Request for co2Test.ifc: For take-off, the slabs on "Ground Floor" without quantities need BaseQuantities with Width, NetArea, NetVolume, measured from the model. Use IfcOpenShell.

First a look at what the model holds.

```python
import ifcopenshell
import ifcopenshell.util.element
import ifcopenshell.util.unit

model = ifcopenshell.open("co2Test.ifc")
print(model.schema)
for unit_type in ("LENGTHUNIT", "AREAUNIT", "VOLUMEUNIT"):
    print(unit_type, ifcopenshell.util.unit.calculate_unit_scale(model, unit_type))
storey = next(s for s in model.by_type("IfcBuildingStorey") if s.Name == "Ground Floor")
slabs = [e for e in ifcopenshell.util.element.get_decomposition(storey) if e.is_a("IfcSlab")]
for e in sorted(slabs, key=lambda e: e.id()):
    print(e.id(), e.is_a(), e.Name, list(ifcopenshell.util.element.get_psets(e, qtos_only=True)), sep=" | ")
```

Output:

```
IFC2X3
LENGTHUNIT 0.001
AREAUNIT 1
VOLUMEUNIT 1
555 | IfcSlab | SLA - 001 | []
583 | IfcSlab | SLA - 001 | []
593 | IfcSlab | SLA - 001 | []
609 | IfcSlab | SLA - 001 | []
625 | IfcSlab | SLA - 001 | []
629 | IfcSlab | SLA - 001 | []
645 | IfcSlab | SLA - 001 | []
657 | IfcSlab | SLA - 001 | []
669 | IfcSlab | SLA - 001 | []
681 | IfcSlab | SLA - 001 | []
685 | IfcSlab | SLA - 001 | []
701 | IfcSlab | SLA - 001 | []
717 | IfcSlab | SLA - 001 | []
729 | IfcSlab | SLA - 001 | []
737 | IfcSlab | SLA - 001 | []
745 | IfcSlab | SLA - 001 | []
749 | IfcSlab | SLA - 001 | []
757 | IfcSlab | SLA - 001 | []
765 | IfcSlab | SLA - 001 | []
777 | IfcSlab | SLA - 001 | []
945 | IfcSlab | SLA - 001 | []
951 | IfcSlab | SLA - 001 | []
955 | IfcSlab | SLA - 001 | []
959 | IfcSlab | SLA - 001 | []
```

```python
import ifcopenshell
import ifcopenshell.api.pset
import ifcopenshell.geom
import ifcopenshell.util.element
import ifcopenshell.util.shape
import ifcopenshell.util.unit

model = ifcopenshell.open("co2Test.ifc")
unit_scale = ifcopenshell.util.unit.calculate_unit_scale(model)
area_scale = ifcopenshell.util.unit.calculate_unit_scale(model, "AREAUNIT")
volume_scale = ifcopenshell.util.unit.calculate_unit_scale(model, "VOLUMEUNIT")
settings = ifcopenshell.geom.settings()

storey = next(s for s in model.by_type("IfcBuildingStorey") if s.Name == "Ground Floor")
slabs = [e for e in ifcopenshell.util.element.get_decomposition(storey) if e.is_a("IfcSlab")]

for e in sorted(slabs, key=lambda e: e.id()):
    if ifcopenshell.util.element.get_psets(e, qtos_only=True, should_inherit=False):
        continue
    # Geometry comes back in metres, in the element's own axes.
    shape = ifcopenshell.geom.create_shape(settings, e)
    values = {
        "Width": ifcopenshell.util.shape.get_z(shape.geometry) / unit_scale,
        "NetArea": ifcopenshell.util.shape.get_footprint_area(shape.geometry) / area_scale,
        "NetVolume": ifcopenshell.util.shape.get_volume(shape.geometry) / volume_scale,
    }
    qto = ifcopenshell.api.pset.add_qto(model, product=e, name="BaseQuantities")
    ifcopenshell.api.pset.edit_qto(model, qto=qto, properties=values)
    print(e.id(), {k: round(v, 3) for k, v in values.items()})

model.write("co2Test_rev.ifc")
```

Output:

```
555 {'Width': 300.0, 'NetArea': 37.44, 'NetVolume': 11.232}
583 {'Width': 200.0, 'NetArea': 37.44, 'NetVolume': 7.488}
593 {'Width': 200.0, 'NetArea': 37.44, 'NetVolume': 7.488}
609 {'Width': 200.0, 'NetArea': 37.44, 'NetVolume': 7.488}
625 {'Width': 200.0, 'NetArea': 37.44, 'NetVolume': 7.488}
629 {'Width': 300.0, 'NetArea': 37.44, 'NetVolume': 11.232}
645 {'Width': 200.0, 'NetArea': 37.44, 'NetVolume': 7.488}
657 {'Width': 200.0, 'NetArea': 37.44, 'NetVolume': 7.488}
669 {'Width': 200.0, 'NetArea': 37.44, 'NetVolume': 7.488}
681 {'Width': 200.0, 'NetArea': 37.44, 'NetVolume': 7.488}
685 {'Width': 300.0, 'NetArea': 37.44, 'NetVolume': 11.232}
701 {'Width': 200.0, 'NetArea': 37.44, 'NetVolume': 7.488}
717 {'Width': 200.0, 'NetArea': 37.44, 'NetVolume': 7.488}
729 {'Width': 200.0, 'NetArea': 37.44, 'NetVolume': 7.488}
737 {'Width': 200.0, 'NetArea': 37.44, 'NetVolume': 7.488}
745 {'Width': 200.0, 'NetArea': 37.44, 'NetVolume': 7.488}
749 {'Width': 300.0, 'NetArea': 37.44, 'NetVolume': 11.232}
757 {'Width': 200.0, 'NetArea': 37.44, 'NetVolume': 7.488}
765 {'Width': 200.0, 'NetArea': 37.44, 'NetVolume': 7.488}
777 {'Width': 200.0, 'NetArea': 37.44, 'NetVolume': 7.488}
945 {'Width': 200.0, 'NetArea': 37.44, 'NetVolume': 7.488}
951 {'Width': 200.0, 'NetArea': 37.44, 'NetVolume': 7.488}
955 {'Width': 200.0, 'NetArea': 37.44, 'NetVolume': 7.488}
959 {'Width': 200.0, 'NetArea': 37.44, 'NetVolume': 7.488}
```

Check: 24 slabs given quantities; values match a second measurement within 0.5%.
